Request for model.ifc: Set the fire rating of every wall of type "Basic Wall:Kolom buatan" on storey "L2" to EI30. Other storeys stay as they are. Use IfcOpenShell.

First a look at what the model holds.

```python
import ifcopenshell
import ifcopenshell.util.element

model = ifcopenshell.open("model.ifc")
print(model.schema)
storey = next(s for s in model.by_type("IfcBuildingStorey") if s.Name == "L2")
walls = [e for e in ifcopenshell.util.element.get_decomposition(storey) if e.is_a("IfcWall")]
seen = {}
for e in walls:
    element_type = ifcopenshell.util.element.get_type(e)
    key = (element_type.Name if element_type != e and element_type else None, ifcopenshell.util.element.get_pset(e, "Pset_WallCommon", "FireRating"))
    seen[key] = seen.get(key, 0) + 1
for (name, value), count in sorted(seen.items(), key=str):
    print(count, "x", name, "|", value)
```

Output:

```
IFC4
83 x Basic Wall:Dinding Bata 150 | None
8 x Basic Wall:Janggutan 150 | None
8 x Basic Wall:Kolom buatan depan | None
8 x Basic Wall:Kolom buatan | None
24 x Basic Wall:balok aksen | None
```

```python
import ifcopenshell
import ifcopenshell.api.pset
import ifcopenshell.util.element

model = ifcopenshell.open("model.ifc")

storey = next(s for s in model.by_type("IfcBuildingStorey") if s.Name == "L2")
walls = [e for e in ifcopenshell.util.element.get_decomposition(storey) if e.is_a("IfcWall")]

count = 0
for e in walls:
    element_type = ifcopenshell.util.element.get_type(e)
    if element_type in (None, e) or element_type.Name != "Basic Wall:Kolom buatan":
        continue
    # add_pset returns the element's existing set when there is one.
    pset = ifcopenshell.api.pset.add_pset(model, product=e, name="Pset_WallCommon")
    ifcopenshell.api.pset.edit_pset(model, pset=pset, properties={"FireRating": "EI30"})
    count += 1

print(count, "walls updated")

model.write("model_v2.ifc")
```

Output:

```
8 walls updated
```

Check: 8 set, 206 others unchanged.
